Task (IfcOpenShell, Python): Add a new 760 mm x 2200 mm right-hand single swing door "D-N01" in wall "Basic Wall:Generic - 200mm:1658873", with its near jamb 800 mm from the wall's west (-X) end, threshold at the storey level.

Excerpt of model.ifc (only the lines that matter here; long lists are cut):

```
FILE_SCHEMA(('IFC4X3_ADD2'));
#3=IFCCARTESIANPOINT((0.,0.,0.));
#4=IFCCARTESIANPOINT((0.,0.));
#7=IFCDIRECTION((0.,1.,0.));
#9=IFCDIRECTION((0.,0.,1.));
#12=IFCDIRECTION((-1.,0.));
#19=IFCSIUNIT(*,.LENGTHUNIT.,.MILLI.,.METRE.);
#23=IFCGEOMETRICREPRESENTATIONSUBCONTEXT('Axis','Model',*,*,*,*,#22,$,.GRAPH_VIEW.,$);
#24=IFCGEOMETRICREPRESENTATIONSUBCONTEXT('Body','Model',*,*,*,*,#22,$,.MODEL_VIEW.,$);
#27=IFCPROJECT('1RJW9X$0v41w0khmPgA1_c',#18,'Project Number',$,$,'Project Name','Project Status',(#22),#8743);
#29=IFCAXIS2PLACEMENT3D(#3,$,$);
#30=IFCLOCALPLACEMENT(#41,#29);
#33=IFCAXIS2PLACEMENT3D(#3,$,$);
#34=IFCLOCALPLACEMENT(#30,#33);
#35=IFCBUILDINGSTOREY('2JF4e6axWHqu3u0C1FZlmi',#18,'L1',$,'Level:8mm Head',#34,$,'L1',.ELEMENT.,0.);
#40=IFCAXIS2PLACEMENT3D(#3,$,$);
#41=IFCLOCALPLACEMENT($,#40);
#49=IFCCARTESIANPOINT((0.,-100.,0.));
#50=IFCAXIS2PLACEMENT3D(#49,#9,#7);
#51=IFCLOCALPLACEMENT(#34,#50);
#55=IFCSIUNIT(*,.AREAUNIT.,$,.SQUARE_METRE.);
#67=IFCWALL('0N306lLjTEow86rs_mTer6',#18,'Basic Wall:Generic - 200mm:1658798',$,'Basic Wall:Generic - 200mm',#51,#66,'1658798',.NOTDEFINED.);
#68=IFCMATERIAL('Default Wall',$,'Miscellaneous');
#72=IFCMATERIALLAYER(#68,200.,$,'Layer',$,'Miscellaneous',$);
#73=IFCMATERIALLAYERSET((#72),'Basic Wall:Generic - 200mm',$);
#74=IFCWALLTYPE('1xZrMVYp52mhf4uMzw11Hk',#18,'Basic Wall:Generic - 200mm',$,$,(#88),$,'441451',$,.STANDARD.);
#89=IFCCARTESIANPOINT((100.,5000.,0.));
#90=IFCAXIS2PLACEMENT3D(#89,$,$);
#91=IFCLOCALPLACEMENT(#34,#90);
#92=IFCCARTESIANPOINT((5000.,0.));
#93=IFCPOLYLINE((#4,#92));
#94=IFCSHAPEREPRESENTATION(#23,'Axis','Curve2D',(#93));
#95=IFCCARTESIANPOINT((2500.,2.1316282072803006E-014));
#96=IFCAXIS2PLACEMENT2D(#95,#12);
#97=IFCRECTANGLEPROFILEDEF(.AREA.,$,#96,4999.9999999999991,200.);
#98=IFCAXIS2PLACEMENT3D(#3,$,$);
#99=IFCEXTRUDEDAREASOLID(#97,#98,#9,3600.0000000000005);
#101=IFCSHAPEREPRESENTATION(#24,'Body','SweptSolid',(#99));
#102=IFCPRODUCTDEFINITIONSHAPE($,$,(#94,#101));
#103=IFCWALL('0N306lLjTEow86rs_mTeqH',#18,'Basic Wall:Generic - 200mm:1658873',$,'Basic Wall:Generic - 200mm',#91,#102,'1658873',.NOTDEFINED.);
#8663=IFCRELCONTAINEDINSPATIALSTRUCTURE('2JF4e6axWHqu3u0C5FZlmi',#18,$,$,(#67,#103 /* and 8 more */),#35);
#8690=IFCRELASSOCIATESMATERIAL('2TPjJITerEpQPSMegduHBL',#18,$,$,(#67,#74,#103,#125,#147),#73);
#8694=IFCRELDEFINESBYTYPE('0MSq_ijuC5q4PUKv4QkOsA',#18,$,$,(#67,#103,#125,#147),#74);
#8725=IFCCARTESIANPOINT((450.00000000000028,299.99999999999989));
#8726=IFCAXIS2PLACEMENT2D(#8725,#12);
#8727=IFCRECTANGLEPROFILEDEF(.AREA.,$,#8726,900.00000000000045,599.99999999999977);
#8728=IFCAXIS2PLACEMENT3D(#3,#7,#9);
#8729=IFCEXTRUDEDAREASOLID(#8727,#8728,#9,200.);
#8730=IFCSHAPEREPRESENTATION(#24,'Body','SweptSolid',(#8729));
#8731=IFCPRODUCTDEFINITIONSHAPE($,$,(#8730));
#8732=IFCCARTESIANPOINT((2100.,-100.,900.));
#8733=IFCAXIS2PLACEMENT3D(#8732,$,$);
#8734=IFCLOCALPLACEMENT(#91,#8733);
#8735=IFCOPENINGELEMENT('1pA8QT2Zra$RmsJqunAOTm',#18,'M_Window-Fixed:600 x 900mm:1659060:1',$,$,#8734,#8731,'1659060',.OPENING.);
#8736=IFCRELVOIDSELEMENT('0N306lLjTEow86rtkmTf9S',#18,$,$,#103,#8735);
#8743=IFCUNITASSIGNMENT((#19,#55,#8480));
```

```python
import numpy as np
import ifcopenshell
import ifcopenshell.api.feature
import ifcopenshell.api.geometry
import ifcopenshell.api.root
import ifcopenshell.api.spatial
import ifcopenshell.geom
import ifcopenshell.util.element
import ifcopenshell.util.placement
import ifcopenshell.util.representation
import ifcopenshell.util.shape
import ifcopenshell.util.unit

model = ifcopenshell.open("model.ifc")
unit_scale = ifcopenshell.util.unit.calculate_unit_scale(model)
settings = ifcopenshell.geom.settings()


def volume(element):
    """Net volume in cubic metres, openings subtracted."""
    shape = ifcopenshell.geom.create_shape(settings, element)
    return ifcopenshell.util.shape.get_volume(shape.geometry)


wall = model.by_id(103)
storey = ifcopenshell.util.element.get_container(wall, ifc_class="IfcBuildingStorey")
context = ifcopenshell.util.representation.get_context(model, "Model", "Body", "MODEL_VIEW")
before = volume(wall)

width, height, from_end, sill = 0.76, 2.2, 0.8, 0.0  # metres

# The wall runs along its own X axis, and the end named is its -X end.
wall_shape = ifcopenshell.geom.create_shape(settings, wall)
x, y, z = ifcopenshell.util.shape.get_vertices(wall_shape.geometry).T
start = x.min() + from_end
face, thickness = float(y.min()), float(y.max() - y.min())
wall_matrix = ifcopenshell.util.placement.get_local_placement(wall.ObjectPlacement)
level = ifcopenshell.util.placement.get_local_placement(storey.ObjectPlacement)[2, 3]


def in_wall(x, y):
    """Placement at x, y metres in the wall's axes, at sill height."""
    matrix = wall_matrix.copy()
    matrix[:, 3] = wall_matrix @ np.array([x / unit_scale, y / unit_scale, 0.0, 1.0])
    matrix[2, 3] = level + sill / unit_scale
    return matrix


# Opening: a box that overshoots both wall faces by 50 mm.
opening = ifcopenshell.api.root.create_entity(model, ifc_class="IfcOpeningElement", predefined_type="OPENING")
box = ifcopenshell.api.geometry.add_wall_representation(
    model, context=context, length=width, height=height, thickness=thickness + 0.1
)
ifcopenshell.api.geometry.assign_representation(model, product=opening, representation=box)
ifcopenshell.api.geometry.edit_object_placement(model, product=opening, matrix=in_wall(start, face - 0.05), is_si=False)
ifcopenshell.api.feature.add_feature(model, feature=opening, element=wall)

door = ifcopenshell.api.root.create_entity(model, ifc_class="IfcDoor", name="D-N01", predefined_type="DOOR")
door.OverallWidth, door.OverallHeight = width / unit_scale, height / unit_scale
door.OperationType = "SINGLE_SWING_RIGHT"
body = ifcopenshell.api.geometry.add_door_representation(
    model,
    context=context,
    overall_width=door.OverallWidth,
    overall_height=door.OverallHeight,
    operation_type="SINGLE_SWING_RIGHT",
    lining_properties={"LiningDepth": thickness / unit_scale, "ThresholdDepth": thickness / unit_scale},
)
ifcopenshell.api.geometry.assign_representation(model, product=door, representation=body)
ifcopenshell.api.spatial.assign_container(model, products=[door], relating_structure=storey)
ifcopenshell.api.feature.add_filling(model, opening=opening, element=door)

# The lining spans the wall, so the door starts at the wall face.
ifcopenshell.api.geometry.edit_object_placement(model, product=door, matrix=in_wall(start, face), is_si=False)

after = volume(wall)

print(f"wall volume {before:.3f} -> {after:.3f} m3")

model.write("model_v2.ifc")
```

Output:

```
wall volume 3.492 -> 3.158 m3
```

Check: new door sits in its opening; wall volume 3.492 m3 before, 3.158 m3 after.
